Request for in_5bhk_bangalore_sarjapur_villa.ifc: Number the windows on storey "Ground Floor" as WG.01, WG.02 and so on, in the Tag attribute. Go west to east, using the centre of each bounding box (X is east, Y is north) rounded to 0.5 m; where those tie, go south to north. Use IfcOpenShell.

First a look at what the model holds.

```python
import ifcopenshell
import ifcopenshell.util.element
import ifcopenshell.util.placement

model = ifcopenshell.open("in_5bhk_bangalore_sarjapur_villa.ifc")
print(model.schema)
storey = next(s for s in model.by_type("IfcBuildingStorey") if s.Name == "Ground Floor")
windows = [e for e in ifcopenshell.util.element.get_decomposition(storey) if e.is_a("IfcWindow")]
for e in sorted(windows, key=lambda e: e.id()):
    origin = ifcopenshell.util.placement.get_local_placement(e.ObjectPlacement)[:3, 3]
    print(e.id(), e.Tag, e.Name, origin.round(2) + 0.0, sep=" | ")
```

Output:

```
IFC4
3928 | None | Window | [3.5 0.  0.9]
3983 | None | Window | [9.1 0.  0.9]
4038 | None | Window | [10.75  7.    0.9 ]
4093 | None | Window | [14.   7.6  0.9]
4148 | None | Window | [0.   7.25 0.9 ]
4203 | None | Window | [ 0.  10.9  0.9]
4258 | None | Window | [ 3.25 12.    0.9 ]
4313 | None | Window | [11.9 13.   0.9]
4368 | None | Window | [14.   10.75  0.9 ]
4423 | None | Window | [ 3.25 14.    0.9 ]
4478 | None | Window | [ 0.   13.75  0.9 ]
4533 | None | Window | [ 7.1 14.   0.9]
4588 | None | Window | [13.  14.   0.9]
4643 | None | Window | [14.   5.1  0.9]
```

```python
import ifcopenshell
import ifcopenshell.geom
import ifcopenshell.util.element
import ifcopenshell.util.shape

model = ifcopenshell.open("in_5bhk_bangalore_sarjapur_villa.ifc")
settings = ifcopenshell.geom.settings()
settings.set("use-world-coords", True)


def centre(element):
    shape = ifcopenshell.geom.create_shape(settings, element)
    return ifcopenshell.util.shape.get_bbox_centroid(shape.geometry)


storey = next(s for s in model.by_type("IfcBuildingStorey") if s.Name == "Ground Floor")
windows = [e for e in ifcopenshell.util.element.get_decomposition(storey) if e.is_a("IfcWindow")]

# Insertion points can sit at a corner or the storey origin, so sort by the geometry (in metres).
centres = {e: centre(e) for e in windows}
windows.sort(key=lambda e: (round(centres[e][0] / 0.5), centres[e][1]))

for i, e in enumerate(windows, start=1):
    number = f"WG.{i:02d}"
    e.Tag = number
    print(e.id(), number)

model.write("in_5bhk_bangalore_sarjapur_villa_rev.ifc")
```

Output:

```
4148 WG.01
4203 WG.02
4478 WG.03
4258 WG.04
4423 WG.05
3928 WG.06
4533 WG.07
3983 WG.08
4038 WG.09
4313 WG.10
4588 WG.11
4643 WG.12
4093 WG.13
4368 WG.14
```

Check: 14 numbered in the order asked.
